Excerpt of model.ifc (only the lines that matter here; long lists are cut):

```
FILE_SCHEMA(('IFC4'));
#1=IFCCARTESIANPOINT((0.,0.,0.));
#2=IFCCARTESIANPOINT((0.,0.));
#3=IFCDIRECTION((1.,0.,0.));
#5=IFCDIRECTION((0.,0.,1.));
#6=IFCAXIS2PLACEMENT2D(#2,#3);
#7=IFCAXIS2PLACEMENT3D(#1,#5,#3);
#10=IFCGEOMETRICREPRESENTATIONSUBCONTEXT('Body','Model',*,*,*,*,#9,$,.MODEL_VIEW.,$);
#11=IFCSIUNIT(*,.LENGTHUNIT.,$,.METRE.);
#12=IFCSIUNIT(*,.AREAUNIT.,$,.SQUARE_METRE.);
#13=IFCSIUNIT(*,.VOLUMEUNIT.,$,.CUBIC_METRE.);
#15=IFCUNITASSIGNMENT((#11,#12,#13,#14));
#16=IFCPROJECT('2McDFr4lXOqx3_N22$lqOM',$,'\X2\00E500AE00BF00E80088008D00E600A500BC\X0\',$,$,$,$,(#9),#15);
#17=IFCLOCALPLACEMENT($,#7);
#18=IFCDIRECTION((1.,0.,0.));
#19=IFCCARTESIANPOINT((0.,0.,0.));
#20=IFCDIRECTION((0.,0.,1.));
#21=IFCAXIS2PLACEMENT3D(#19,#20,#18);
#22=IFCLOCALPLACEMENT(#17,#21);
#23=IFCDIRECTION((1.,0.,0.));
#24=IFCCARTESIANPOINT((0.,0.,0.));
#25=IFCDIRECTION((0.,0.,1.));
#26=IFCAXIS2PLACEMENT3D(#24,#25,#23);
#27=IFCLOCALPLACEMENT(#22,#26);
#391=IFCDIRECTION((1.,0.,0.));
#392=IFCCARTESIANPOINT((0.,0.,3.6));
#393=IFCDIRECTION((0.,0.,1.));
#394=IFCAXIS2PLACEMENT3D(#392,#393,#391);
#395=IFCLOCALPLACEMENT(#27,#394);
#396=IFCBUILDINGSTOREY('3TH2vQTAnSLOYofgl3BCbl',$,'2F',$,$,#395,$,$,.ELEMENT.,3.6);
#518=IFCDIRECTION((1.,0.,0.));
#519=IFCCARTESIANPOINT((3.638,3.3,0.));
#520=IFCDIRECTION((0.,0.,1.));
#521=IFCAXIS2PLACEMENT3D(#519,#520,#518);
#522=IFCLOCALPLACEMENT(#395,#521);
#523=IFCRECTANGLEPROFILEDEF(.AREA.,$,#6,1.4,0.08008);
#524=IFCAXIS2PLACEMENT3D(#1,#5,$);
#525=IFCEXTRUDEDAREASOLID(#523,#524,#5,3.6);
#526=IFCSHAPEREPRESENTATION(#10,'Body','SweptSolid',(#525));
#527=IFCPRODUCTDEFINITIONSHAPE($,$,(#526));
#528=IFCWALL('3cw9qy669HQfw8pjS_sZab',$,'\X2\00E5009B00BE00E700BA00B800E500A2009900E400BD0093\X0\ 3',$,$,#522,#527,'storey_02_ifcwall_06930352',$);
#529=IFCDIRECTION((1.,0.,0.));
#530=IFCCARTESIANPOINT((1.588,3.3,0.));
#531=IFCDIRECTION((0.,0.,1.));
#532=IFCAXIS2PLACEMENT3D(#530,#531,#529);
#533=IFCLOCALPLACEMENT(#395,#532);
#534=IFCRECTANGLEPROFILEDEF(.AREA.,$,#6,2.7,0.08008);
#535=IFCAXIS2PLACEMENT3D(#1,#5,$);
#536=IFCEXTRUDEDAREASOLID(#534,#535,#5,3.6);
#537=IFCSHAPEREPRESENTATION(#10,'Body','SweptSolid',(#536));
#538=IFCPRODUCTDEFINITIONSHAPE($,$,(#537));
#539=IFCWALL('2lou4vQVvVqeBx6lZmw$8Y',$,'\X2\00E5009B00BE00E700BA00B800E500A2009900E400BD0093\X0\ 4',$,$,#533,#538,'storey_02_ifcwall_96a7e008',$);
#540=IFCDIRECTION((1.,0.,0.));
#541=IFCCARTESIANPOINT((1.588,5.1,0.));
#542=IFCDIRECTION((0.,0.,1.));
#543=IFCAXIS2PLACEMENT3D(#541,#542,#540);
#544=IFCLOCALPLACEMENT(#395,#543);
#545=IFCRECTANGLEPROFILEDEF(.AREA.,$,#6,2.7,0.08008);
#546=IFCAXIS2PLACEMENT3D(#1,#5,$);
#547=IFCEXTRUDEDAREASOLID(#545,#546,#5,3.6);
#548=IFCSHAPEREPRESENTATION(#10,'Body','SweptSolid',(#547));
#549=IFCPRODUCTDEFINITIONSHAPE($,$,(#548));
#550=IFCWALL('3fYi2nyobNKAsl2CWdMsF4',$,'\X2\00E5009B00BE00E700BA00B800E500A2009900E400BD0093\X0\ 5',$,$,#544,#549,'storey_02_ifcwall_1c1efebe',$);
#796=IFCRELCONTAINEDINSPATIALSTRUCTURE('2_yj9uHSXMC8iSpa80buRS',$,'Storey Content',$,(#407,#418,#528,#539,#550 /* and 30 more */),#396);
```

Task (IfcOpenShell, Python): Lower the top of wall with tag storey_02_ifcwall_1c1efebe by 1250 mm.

```python
import ifcopenshell
import ifcopenshell.geom
import ifcopenshell.util.representation
import ifcopenshell.util.shape
import ifcopenshell.util.unit

model = ifcopenshell.open("model.ifc")
unit_scale = ifcopenshell.util.unit.calculate_unit_scale(model)
settings = ifcopenshell.geom.settings()


def volume(element):
    """Net volume in cubic metres, openings subtracted."""
    shape = ifcopenshell.geom.create_shape(settings, element)
    return ifcopenshell.util.shape.get_volume(shape.geometry)


wall = model.by_guid("3fYi2nyobNKAsl2CWdMsF4")
before = volume(wall)

body = ifcopenshell.util.representation.get_representation(wall, "Model", "Body")
solid = body.Items[0]
old_height = solid.Depth
solid.Depth -= 1.25 / unit_scale
after = volume(wall)

print(f"height {old_height:g} -> {solid.Depth:g}, volume {before:.3f} -> {after:.3f} m3")

model.write("model_edited.ifc")
```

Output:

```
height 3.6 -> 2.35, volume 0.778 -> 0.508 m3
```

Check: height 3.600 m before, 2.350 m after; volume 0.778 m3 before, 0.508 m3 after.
